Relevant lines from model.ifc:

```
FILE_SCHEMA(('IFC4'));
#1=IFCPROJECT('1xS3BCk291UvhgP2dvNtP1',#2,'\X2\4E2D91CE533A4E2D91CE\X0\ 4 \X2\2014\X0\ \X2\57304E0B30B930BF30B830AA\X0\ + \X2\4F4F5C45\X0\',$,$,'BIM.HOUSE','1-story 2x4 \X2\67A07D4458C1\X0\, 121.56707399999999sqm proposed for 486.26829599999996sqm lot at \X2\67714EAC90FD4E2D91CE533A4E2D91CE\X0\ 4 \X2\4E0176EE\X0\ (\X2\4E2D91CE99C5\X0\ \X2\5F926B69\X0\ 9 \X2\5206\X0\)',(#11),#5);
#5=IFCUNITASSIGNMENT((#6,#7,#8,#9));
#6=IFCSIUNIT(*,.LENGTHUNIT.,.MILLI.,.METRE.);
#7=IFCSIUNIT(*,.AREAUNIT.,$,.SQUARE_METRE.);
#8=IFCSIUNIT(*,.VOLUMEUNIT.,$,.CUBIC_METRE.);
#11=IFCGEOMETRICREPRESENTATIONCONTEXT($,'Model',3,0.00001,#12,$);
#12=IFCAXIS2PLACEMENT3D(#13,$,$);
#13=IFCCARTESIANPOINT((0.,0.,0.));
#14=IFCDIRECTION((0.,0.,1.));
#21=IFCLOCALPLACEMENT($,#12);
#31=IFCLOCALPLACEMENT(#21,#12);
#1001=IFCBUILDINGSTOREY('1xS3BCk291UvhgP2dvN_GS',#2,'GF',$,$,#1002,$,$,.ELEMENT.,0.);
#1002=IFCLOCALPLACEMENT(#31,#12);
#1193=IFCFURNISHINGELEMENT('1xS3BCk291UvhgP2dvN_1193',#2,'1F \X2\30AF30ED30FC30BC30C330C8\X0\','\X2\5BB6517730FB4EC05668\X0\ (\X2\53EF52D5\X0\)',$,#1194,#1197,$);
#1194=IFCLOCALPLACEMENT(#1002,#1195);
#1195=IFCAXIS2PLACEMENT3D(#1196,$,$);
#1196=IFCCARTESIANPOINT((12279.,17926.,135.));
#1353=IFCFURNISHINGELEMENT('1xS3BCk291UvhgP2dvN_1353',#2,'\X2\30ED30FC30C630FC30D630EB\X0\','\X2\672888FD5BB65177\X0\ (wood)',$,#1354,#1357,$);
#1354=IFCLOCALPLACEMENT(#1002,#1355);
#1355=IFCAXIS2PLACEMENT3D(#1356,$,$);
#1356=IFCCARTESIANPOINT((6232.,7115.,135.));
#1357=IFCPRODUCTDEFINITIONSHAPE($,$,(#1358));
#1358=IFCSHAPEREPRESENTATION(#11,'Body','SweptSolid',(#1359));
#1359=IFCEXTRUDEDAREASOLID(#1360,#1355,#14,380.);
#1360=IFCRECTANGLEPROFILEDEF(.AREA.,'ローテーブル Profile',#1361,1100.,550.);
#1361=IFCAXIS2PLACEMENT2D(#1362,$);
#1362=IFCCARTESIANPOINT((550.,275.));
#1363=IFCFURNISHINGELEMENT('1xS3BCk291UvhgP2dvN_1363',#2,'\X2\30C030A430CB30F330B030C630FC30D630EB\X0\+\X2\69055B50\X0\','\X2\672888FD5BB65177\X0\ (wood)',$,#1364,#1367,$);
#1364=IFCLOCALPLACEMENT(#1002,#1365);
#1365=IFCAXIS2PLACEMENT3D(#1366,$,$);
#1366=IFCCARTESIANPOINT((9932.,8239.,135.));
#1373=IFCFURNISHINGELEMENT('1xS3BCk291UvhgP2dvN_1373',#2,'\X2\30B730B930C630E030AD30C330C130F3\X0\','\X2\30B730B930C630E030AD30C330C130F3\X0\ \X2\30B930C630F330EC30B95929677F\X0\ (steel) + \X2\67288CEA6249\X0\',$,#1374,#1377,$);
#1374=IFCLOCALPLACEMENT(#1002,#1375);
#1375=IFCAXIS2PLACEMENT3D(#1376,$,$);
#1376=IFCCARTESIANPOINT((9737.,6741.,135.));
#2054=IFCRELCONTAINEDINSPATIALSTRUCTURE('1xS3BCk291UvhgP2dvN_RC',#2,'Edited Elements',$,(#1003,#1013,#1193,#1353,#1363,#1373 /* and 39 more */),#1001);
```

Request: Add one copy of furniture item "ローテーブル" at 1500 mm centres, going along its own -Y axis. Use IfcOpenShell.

```python
import ifcopenshell
import ifcopenshell.api.geometry
import ifcopenshell.api.root
import ifcopenshell.util.element
import ifcopenshell.util.placement
import ifcopenshell.util.unit

model = ifcopenshell.open("model.ifc")
unit_scale = ifcopenshell.util.unit.calculate_unit_scale(model)


def reuse_history(source, copy):
    """copy_class also copies each property set's owner history, people and application; keep the originals."""
    for rel in copy.IsDefinedBy:
        if rel.is_a("IfcRelDefinesByProperties") and (history := rel.RelatingPropertyDefinition.OwnerHistory):
            rel.RelatingPropertyDefinition.OwnerHistory = source.OwnerHistory
            ifcopenshell.util.element.remove_deep2(model, history)


source = model.by_guid("1xS3BCk291UvhgP2dvN_1353")
base = ifcopenshell.util.placement.get_local_placement(source.ObjectPlacement)
step = -base[:3, 1] * 1.5 / unit_scale

for i in range(1, 2):
    copy = ifcopenshell.api.root.copy_class(model, product=source)
    copy.Representation = ifcopenshell.util.element.copy_deep(
        model, source.Representation, exclude=["IfcGeometricRepresentationContext", "IfcRepresentationMap"]
    )
    reuse_history(source, copy)
    matrix = base.copy()
    matrix[:3, 3] += i * step
    print("added at", matrix[:3, 3].round(3) + 0.0)
    ifcopenshell.api.geometry.edit_object_placement(model, product=copy, matrix=matrix, is_si=False)

model.write("model_updated.ifc")
```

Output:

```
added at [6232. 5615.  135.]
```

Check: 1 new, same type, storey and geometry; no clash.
